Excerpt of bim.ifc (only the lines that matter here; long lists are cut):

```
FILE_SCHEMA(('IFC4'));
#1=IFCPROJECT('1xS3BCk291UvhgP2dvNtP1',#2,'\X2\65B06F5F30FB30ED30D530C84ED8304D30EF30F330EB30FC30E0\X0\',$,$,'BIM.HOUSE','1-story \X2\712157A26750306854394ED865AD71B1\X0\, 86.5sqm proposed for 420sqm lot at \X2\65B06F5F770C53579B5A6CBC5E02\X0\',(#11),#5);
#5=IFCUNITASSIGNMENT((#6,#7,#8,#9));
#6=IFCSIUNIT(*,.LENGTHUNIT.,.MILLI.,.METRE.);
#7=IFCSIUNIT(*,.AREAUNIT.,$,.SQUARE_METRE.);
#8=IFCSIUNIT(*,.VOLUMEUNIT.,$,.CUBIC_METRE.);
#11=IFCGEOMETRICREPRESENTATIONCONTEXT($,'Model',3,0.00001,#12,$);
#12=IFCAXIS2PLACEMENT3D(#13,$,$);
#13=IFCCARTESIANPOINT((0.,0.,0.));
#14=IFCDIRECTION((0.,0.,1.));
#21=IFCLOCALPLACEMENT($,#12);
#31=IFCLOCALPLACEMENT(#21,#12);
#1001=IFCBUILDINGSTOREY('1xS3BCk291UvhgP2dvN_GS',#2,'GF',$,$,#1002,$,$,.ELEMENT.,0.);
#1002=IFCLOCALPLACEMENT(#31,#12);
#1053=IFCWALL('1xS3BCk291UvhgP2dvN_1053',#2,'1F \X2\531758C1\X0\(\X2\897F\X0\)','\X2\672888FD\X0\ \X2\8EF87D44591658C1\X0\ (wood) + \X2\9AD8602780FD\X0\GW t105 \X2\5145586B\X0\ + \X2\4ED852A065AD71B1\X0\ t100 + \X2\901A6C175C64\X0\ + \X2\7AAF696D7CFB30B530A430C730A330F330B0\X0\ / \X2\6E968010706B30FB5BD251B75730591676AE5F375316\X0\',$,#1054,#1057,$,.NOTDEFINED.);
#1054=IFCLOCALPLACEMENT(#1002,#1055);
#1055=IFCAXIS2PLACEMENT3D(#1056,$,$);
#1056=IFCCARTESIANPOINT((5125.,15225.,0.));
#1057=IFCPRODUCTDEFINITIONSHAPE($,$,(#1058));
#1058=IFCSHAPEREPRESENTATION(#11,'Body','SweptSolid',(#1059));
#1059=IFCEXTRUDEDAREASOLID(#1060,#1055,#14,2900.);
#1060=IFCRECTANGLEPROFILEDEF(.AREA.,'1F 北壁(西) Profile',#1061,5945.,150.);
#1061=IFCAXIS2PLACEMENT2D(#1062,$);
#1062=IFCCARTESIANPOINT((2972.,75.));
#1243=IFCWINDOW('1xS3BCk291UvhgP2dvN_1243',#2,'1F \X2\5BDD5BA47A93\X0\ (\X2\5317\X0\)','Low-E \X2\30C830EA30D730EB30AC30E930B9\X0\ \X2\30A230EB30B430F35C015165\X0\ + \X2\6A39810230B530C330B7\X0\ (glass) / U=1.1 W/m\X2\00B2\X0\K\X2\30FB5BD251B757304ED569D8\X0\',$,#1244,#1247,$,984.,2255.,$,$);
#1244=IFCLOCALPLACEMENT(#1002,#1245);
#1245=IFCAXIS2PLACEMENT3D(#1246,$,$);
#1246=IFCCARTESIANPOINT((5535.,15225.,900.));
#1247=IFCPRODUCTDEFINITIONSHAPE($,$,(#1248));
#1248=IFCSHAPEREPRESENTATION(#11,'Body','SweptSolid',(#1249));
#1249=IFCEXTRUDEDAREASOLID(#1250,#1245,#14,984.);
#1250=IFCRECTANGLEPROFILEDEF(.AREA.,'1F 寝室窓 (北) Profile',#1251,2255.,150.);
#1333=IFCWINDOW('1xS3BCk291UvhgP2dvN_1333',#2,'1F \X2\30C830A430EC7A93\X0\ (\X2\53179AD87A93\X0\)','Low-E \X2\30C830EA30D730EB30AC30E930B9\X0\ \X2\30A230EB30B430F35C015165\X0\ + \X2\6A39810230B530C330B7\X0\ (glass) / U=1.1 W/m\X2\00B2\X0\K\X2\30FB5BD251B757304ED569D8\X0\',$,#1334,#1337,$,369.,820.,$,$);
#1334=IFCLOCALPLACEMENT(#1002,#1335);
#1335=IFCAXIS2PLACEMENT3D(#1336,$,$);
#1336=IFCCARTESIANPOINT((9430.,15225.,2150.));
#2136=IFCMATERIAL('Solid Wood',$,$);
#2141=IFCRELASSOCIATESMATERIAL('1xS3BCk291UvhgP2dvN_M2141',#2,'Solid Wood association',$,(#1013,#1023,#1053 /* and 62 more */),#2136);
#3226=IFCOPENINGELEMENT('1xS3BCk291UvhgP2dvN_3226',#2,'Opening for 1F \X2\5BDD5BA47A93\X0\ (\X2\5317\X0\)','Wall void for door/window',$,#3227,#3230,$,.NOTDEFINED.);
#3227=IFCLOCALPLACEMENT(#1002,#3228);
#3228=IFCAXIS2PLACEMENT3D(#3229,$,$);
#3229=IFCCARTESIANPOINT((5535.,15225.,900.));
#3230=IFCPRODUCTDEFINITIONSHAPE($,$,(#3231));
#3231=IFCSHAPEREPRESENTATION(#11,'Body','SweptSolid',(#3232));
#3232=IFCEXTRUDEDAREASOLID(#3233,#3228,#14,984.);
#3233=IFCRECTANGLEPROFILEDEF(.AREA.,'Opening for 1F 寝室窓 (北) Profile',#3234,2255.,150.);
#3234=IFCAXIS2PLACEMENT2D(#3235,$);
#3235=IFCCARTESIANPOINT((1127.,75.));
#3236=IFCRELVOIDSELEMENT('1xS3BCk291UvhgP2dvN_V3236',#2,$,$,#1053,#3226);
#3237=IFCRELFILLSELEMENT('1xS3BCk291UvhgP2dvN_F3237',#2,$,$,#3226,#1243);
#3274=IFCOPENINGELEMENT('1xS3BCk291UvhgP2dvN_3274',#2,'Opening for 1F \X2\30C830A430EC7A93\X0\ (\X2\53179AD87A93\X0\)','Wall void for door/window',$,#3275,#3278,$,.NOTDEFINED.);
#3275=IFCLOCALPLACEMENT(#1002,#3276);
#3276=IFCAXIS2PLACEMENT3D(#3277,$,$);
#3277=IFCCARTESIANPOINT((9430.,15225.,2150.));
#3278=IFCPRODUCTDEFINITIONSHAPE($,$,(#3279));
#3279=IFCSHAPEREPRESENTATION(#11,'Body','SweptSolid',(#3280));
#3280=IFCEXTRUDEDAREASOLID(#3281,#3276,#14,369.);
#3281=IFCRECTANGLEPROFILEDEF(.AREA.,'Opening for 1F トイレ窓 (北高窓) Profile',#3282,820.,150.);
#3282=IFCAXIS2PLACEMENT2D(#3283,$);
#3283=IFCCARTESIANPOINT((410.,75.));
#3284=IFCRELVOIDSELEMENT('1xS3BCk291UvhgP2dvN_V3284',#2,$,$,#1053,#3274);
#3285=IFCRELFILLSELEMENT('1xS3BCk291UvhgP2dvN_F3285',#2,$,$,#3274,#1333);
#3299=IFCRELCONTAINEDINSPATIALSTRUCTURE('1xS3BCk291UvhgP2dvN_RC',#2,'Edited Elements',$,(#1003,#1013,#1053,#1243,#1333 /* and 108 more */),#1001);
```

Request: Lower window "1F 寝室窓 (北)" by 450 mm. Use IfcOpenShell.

```python
import numpy as np
import ifcopenshell
import ifcopenshell.api.geometry
import ifcopenshell.util.placement
import ifcopenshell.util.unit

model = ifcopenshell.open("bim.ifc")
unit_scale = ifcopenshell.util.unit.calculate_unit_scale(model)

window = model.by_id(1243)
opening = window.FillsVoids[0].RelatingOpeningElement
dz = -0.45 / unit_scale

shift = np.array([0.0, 0.0, dz])
# The window is not placed relative to its opening, so move both.
for product in (opening, window):
    matrix = ifcopenshell.util.placement.get_local_placement(product.ObjectPlacement)
    matrix[:3, 3] += shift
    ifcopenshell.api.geometry.edit_object_placement(model, product=product, matrix=matrix, is_si=False)

print(f"moved by {dz * unit_scale:+.3f} m")

model.write("bim-out.ifc")
```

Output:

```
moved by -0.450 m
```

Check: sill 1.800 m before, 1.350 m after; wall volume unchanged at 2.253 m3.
